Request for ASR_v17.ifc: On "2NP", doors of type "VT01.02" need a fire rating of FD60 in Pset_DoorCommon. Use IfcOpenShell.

First a look at what the model holds.

```python
import ifcopenshell
import ifcopenshell.util.element

model = ifcopenshell.open("ASR_v17.ifc")
print(model.schema)
storey = next(s for s in model.by_type("IfcBuildingStorey") if s.Name == "2NP")
doors = [e for e in ifcopenshell.util.element.get_decomposition(storey) if e.is_a("IfcDoor")]
seen = {}
for e in doors:
    element_type = ifcopenshell.util.element.get_type(e)
    key = (element_type.Name if element_type != e and element_type else None, ifcopenshell.util.element.get_pset(e, "Pset_DoorCommon", "FireRating"))
    seen[key] = seen.get(key, 0) + 1
for (name, value), count in sorted(seen.items(), key=str):
    print(count, "x", name, "|", value)
```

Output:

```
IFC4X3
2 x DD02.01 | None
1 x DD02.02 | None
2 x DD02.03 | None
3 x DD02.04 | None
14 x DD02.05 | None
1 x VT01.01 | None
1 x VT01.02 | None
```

```python
import ifcopenshell
import ifcopenshell.api.pset
import ifcopenshell.util.element

model = ifcopenshell.open("ASR_v17.ifc")

storey = next(s for s in model.by_type("IfcBuildingStorey") if s.Name == "2NP")
doors = [e for e in ifcopenshell.util.element.get_decomposition(storey) if e.is_a("IfcDoor")]

count = 0
for e in doors:
    element_type = ifcopenshell.util.element.get_type(e)
    if element_type in (None, e) or element_type.Name != "VT01.02":
        continue
    # add_pset returns the element's existing set when there is one.
    pset = ifcopenshell.api.pset.add_pset(model, product=e, name="Pset_DoorCommon")
    ifcopenshell.api.pset.edit_pset(model, pset=pset, properties={"FireRating": "FD60"})
    count += 1

print(count, "doors updated")

model.write("ASR_v17_v2.ifc")
```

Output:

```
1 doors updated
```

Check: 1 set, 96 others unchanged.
